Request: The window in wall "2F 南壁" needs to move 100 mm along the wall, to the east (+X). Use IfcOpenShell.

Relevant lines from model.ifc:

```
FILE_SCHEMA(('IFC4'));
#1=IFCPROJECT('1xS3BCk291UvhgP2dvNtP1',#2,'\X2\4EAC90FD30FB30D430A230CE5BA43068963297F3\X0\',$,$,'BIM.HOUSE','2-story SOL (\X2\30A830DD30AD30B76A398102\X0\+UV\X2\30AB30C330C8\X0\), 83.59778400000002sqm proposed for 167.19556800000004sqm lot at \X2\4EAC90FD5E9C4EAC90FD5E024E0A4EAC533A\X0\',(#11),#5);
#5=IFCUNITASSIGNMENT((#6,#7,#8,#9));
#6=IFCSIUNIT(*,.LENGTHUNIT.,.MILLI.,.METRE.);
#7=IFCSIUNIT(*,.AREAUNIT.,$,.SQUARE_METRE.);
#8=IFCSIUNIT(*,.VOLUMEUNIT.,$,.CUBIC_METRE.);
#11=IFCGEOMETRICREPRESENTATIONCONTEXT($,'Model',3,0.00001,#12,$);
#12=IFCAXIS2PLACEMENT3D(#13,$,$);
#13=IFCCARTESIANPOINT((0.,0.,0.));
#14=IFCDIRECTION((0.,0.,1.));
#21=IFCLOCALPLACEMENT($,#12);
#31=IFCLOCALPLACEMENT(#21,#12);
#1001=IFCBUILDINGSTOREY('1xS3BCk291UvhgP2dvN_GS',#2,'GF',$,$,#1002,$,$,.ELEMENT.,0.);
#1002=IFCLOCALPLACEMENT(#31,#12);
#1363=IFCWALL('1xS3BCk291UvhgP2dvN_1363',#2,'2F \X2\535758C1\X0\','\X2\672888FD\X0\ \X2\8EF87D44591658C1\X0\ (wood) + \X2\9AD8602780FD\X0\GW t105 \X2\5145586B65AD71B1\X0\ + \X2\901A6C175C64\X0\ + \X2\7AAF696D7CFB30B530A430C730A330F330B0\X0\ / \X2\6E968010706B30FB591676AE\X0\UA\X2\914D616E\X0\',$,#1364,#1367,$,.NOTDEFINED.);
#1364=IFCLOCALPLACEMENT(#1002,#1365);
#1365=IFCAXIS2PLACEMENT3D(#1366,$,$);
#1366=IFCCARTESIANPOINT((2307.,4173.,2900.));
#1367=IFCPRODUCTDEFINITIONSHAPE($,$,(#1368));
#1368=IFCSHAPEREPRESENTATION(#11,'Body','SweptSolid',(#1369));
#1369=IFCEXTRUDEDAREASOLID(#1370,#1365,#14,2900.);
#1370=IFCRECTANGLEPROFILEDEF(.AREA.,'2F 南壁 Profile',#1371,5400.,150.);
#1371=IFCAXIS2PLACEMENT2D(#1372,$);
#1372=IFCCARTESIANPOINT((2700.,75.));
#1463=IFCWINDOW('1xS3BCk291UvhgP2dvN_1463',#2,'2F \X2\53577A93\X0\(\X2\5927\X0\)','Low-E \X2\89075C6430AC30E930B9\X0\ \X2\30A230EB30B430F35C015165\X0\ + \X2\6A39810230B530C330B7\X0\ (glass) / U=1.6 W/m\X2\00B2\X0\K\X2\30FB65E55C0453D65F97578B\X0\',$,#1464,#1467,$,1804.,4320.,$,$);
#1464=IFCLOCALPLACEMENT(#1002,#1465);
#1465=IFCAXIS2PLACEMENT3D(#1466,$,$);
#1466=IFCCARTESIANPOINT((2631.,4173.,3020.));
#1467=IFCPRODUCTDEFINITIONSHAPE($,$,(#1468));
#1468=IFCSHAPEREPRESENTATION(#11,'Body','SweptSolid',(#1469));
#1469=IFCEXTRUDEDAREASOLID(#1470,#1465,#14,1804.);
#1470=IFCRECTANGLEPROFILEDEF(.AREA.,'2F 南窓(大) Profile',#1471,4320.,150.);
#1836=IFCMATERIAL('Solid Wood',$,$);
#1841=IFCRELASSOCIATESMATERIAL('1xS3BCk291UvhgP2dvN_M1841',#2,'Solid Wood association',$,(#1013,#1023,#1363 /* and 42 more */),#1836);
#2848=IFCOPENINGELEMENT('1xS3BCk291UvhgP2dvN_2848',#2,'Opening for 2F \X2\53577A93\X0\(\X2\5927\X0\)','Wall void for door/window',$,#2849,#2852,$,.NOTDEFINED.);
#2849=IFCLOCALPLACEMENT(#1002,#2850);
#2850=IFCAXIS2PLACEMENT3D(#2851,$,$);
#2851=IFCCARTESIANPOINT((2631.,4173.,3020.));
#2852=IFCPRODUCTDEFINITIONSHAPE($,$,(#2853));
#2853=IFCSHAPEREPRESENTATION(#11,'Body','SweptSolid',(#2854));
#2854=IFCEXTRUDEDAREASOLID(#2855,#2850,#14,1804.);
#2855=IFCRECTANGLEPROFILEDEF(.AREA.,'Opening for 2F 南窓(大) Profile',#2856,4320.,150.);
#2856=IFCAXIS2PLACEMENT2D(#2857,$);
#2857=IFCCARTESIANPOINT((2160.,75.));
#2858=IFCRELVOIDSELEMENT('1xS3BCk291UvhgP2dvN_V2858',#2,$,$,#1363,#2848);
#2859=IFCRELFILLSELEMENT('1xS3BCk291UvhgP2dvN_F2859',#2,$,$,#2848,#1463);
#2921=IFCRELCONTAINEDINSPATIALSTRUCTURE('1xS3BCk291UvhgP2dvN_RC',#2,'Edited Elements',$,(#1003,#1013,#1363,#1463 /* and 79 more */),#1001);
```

```python
import ifcopenshell
import ifcopenshell.api.geometry
import ifcopenshell.util.placement
import ifcopenshell.util.unit

model = ifcopenshell.open("model.ifc")
unit_scale = ifcopenshell.util.unit.calculate_unit_scale(model)

window = model.by_guid("1xS3BCk291UvhgP2dvN_1463")
opening = window.FillsVoids[0].RelatingOpeningElement
wall = opening.VoidsElements[0].RelatingBuildingElement

wall_matrix = ifcopenshell.util.placement.get_local_placement(wall.ObjectPlacement)
shift = wall_matrix[:3, 0] * 0.1 / unit_scale
before = ifcopenshell.util.placement.get_local_placement(window.ObjectPlacement)[:3, 3].copy()

# The window is not placed relative to its opening, so move both.
for product in (opening, window):
    matrix = ifcopenshell.util.placement.get_local_placement(product.ObjectPlacement)
    matrix[:3, 3] += shift
    ifcopenshell.api.geometry.edit_object_placement(model, product=product, matrix=matrix, is_si=False)

after = ifcopenshell.util.placement.get_local_placement(window.ObjectPlacement)[:3, 3]
print("window moved by", (after - before).round(3) + 0.0)

model.write("model_v2.ifc")
```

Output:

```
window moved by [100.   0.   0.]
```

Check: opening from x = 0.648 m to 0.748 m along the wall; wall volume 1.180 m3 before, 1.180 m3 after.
